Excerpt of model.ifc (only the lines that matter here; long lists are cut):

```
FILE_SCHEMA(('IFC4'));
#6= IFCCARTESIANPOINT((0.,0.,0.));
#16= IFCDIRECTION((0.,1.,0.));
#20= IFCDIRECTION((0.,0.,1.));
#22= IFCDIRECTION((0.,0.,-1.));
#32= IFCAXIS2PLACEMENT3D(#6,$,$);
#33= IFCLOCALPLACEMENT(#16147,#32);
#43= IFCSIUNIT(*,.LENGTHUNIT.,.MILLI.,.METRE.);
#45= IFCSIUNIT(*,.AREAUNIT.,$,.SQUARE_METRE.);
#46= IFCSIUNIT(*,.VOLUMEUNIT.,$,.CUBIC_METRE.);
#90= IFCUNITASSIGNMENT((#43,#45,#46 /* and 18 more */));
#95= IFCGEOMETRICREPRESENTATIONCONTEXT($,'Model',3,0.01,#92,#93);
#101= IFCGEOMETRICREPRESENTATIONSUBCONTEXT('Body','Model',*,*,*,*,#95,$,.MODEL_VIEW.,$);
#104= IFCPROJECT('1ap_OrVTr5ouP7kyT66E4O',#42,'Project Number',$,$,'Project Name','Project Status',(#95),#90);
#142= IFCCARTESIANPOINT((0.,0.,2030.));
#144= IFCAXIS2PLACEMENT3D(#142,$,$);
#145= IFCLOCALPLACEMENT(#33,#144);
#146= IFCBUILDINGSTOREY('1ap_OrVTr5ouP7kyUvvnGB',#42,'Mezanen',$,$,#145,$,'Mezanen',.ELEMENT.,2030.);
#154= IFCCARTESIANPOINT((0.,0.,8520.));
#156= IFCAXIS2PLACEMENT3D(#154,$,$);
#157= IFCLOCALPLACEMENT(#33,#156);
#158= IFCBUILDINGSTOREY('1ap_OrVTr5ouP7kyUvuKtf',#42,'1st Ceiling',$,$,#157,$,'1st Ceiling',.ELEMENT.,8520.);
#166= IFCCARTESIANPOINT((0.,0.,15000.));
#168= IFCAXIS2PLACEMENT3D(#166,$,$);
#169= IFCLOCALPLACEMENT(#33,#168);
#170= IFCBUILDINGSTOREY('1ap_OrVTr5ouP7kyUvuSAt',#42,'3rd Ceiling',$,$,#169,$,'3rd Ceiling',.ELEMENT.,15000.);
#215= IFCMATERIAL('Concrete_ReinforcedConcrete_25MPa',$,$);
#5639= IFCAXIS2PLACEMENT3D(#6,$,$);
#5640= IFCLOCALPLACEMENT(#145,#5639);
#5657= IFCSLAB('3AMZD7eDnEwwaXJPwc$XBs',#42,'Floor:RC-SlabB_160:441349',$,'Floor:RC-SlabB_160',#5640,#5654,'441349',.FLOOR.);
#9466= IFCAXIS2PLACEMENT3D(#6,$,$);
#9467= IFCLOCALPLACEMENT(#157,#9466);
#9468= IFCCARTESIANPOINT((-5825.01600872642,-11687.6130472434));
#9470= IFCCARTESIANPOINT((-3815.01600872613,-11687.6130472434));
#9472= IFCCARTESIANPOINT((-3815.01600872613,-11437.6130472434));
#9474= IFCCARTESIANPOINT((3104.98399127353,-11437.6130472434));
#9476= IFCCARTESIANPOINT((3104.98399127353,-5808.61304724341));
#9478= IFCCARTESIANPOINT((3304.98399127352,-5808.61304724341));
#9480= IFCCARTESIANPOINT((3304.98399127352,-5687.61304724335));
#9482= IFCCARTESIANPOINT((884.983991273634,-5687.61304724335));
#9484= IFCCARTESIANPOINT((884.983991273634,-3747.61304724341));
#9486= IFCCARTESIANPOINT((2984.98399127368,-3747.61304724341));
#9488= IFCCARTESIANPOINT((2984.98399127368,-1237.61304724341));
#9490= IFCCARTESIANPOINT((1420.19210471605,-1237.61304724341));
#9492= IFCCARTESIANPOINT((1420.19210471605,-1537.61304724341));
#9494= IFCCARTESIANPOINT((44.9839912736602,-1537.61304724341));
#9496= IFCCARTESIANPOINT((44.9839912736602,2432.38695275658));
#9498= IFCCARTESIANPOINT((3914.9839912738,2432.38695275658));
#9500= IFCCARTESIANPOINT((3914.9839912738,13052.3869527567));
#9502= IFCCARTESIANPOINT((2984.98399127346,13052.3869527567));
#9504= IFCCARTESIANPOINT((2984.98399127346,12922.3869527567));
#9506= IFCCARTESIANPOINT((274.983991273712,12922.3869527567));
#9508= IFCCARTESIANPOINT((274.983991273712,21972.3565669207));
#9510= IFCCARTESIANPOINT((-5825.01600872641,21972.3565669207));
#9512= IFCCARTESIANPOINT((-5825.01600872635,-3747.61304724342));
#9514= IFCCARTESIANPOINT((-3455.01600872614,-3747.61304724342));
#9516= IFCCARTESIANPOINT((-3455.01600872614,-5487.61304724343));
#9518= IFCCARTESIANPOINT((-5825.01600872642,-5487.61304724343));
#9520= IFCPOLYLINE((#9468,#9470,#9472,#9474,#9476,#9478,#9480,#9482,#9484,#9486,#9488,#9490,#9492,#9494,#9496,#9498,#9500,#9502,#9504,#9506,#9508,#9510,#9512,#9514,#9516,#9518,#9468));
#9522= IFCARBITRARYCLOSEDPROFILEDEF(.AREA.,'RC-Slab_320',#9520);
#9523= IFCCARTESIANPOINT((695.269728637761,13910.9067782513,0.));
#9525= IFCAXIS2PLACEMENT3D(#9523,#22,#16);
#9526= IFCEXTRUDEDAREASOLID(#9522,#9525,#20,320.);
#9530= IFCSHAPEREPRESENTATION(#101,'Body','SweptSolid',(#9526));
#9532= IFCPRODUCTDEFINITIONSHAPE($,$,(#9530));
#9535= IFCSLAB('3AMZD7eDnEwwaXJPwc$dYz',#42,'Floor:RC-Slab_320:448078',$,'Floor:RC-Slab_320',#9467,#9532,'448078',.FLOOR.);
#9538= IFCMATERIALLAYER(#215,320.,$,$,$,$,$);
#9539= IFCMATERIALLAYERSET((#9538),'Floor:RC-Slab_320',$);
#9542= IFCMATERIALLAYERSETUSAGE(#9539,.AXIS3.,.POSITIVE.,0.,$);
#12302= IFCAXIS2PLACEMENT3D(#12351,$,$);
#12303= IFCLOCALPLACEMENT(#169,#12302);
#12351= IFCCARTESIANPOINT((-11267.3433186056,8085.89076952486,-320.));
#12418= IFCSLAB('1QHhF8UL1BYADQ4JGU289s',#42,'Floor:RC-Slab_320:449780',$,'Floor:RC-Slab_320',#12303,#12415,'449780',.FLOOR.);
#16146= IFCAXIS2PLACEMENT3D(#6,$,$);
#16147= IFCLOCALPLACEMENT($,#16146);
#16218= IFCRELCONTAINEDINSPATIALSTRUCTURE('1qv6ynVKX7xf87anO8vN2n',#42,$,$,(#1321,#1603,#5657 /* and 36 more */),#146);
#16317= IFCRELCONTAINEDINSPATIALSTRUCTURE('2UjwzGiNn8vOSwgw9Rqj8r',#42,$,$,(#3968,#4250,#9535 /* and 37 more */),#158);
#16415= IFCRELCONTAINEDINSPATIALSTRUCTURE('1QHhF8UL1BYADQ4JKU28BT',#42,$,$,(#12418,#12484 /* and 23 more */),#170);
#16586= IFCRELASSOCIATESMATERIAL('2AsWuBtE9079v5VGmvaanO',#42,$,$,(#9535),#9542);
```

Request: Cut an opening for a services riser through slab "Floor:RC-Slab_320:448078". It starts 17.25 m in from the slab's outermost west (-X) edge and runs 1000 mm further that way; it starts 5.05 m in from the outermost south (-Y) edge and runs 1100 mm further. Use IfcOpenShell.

```python
import numpy as np
import ifcopenshell
import ifcopenshell.api.feature
import ifcopenshell.api.geometry
import ifcopenshell.api.root
import ifcopenshell.geom
import ifcopenshell.util.placement
import ifcopenshell.util.representation
import ifcopenshell.util.shape
import ifcopenshell.util.unit

model = ifcopenshell.open("model.ifc")
unit_scale = ifcopenshell.util.unit.calculate_unit_scale(model)
settings = ifcopenshell.geom.settings()


def volume(element):
    """Net volume in cubic metres, openings subtracted."""
    shape = ifcopenshell.geom.create_shape(settings, element)
    return ifcopenshell.util.shape.get_volume(shape.geometry)


slab = model.by_guid("3AMZD7eDnEwwaXJPwc$dYz")
before = volume(slab)

# Extent in the slab's own axes, in metres. The edges named are its -X and -Y sides.
slab_shape = ifcopenshell.geom.create_shape(settings, slab)
vertices = ifcopenshell.util.shape.get_vertices(slab_shape.geometry)
x_min, y_min, bottom = vertices.min(axis=0)
top = vertices[:, 2].max()

opening = ifcopenshell.api.root.create_entity(model, ifc_class="IfcOpeningElement", name="Services riser opening", predefined_type="OPENING")
context = ifcopenshell.util.representation.get_context(model, "Model", "Body", "MODEL_VIEW")
width, depth = 1, 1.1
outline = [(0.0, 0.0), (width, 0.0), (width, depth), (0.0, depth), (0.0, 0.0)]
# Overshoot both faces by 50 mm so the cut is clean.
shape = ifcopenshell.api.geometry.add_slab_representation(
    model, context=context, depth=top - bottom + 0.1, polyline=outline
)
ifcopenshell.api.geometry.assign_representation(model, product=opening, representation=shape)

matrix = ifcopenshell.util.placement.get_local_placement(slab.ObjectPlacement)
matrix[:, 3] = matrix @ np.append(np.array([x_min + 17.25, y_min + 5.05, bottom - 0.05]) / unit_scale, 1.0)
ifcopenshell.api.geometry.edit_object_placement(model, product=opening, matrix=matrix, is_si=False)
ifcopenshell.api.feature.add_feature(model, feature=opening, element=slab)

after = volume(slab)

print(f"slab volume {before:.3f} -> {after:.3f} m3")

model.write("model_v2.ifc")
```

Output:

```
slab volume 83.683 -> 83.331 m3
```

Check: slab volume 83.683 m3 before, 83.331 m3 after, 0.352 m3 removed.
